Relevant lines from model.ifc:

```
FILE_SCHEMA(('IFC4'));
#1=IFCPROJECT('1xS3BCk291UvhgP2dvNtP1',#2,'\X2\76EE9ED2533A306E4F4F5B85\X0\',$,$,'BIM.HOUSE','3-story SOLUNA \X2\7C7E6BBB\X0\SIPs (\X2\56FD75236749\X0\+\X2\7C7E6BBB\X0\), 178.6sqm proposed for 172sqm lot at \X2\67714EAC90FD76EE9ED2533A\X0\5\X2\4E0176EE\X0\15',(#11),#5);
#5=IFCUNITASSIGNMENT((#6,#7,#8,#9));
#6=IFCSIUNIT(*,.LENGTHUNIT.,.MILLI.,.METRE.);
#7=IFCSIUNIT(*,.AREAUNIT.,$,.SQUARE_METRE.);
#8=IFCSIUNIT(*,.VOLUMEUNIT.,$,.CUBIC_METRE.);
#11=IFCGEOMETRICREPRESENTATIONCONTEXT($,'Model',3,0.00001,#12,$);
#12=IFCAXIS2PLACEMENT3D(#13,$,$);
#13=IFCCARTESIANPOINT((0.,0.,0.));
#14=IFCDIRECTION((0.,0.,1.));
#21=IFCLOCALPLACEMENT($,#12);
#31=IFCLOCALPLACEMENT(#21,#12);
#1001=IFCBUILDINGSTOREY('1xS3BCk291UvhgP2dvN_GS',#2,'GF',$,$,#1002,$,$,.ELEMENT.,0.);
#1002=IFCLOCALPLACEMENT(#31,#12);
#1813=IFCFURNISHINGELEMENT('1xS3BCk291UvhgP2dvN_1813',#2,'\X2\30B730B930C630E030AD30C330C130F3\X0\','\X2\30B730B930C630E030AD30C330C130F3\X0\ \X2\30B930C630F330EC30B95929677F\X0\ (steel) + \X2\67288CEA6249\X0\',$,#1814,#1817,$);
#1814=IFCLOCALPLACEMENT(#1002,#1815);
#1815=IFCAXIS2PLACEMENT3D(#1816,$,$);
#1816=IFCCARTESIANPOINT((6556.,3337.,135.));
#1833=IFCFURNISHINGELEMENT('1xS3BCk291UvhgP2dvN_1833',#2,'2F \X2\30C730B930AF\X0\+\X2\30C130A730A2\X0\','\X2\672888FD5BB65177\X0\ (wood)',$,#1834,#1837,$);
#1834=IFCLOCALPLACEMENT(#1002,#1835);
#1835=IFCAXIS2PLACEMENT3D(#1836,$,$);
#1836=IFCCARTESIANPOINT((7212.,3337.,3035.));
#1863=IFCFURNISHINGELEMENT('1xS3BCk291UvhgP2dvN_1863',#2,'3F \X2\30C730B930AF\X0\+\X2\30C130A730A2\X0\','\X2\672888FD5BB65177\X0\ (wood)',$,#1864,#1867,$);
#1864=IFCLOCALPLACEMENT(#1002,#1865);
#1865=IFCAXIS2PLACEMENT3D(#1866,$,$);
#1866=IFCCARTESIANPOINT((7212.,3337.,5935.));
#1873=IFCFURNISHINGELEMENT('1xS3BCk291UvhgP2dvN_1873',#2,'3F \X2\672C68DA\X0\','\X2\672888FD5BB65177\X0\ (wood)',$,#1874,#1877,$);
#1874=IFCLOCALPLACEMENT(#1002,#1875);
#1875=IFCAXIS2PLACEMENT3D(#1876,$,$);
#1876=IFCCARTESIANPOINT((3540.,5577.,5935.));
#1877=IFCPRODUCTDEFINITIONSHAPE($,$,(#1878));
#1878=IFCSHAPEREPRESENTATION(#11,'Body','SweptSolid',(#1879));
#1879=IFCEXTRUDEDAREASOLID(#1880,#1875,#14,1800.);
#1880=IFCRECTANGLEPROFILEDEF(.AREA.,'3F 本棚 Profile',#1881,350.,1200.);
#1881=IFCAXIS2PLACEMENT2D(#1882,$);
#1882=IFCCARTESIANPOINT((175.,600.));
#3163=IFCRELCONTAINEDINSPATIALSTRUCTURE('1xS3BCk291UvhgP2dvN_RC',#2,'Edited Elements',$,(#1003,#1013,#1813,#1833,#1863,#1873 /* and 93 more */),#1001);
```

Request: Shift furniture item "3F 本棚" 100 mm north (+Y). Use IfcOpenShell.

```python
import ifcopenshell
import ifcopenshell.api.geometry
import ifcopenshell.util.placement
import ifcopenshell.util.unit

model = ifcopenshell.open("model.ifc")
unit_scale = ifcopenshell.util.unit.calculate_unit_scale(model)

item = model.by_guid("1xS3BCk291UvhgP2dvN_1873")
matrix = ifcopenshell.util.placement.get_local_placement(item.ObjectPlacement)
matrix[1, 3] += 0.1 / unit_scale
ifcopenshell.api.geometry.edit_object_placement(model, product=item, matrix=matrix, is_si=False)

print(ifcopenshell.util.placement.get_local_placement(item.ObjectPlacement).round(3) + 0.0)

model.write("model_updated.ifc")
```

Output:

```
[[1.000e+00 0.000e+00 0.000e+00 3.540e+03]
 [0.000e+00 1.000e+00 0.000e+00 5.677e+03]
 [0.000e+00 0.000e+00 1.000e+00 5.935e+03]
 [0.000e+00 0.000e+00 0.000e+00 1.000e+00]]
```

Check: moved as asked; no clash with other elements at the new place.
